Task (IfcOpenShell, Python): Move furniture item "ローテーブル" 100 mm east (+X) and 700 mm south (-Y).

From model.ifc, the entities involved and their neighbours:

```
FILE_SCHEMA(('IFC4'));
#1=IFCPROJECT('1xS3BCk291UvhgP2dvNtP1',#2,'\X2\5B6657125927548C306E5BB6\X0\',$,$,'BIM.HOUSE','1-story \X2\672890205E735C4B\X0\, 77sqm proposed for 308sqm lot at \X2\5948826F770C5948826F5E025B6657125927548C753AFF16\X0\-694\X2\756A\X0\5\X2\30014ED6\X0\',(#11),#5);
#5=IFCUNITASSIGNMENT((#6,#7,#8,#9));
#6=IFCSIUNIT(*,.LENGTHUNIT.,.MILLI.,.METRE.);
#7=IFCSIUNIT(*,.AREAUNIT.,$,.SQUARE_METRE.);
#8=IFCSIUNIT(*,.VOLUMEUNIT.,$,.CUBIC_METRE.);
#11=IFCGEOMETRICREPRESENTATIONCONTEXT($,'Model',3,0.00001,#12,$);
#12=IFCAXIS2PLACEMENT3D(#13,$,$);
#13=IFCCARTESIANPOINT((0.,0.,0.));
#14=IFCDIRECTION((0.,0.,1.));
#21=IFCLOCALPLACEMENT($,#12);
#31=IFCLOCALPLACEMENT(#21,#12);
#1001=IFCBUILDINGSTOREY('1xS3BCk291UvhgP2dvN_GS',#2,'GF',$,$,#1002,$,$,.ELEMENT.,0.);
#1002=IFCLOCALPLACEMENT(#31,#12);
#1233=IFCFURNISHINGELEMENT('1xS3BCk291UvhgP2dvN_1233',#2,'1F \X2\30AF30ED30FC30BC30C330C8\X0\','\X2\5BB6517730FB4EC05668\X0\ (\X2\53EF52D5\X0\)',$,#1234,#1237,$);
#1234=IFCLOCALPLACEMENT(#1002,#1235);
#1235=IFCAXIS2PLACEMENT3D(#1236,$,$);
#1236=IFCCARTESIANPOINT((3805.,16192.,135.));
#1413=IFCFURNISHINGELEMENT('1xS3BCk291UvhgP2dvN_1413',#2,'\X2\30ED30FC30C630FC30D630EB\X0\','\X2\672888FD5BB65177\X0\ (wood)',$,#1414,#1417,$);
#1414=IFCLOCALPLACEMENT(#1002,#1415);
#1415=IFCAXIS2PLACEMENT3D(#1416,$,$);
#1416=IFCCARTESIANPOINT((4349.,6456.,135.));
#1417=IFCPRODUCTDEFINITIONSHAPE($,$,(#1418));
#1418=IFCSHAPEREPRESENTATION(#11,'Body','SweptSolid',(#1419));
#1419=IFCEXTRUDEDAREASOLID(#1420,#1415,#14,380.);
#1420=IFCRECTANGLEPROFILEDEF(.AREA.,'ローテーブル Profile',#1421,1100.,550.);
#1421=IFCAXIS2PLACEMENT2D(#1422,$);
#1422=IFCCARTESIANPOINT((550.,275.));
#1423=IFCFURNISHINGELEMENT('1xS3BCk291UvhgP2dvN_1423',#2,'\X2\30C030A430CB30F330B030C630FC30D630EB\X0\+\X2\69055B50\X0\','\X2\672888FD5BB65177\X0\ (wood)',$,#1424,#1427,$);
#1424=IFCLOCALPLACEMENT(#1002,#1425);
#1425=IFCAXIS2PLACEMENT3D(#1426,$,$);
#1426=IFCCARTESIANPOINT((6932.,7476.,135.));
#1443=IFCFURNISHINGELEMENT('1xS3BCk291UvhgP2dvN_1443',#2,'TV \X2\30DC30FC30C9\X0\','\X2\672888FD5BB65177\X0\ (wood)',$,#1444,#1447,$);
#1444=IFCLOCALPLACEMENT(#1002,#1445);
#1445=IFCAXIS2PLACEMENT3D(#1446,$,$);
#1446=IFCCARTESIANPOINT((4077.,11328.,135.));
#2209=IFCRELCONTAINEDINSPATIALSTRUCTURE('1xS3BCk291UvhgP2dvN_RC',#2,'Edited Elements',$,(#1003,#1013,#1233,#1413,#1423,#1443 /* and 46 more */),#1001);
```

```python
import ifcopenshell
import ifcopenshell.api.geometry
import ifcopenshell.util.placement
import ifcopenshell.util.unit

model = ifcopenshell.open("model.ifc")
unit_scale = ifcopenshell.util.unit.calculate_unit_scale(model)

item = model.by_guid("1xS3BCk291UvhgP2dvN_1413")
matrix = ifcopenshell.util.placement.get_local_placement(item.ObjectPlacement)
matrix[0, 3] += 0.1 / unit_scale
matrix[1, 3] -= 0.7 / unit_scale
ifcopenshell.api.geometry.edit_object_placement(model, product=item, matrix=matrix, is_si=False)

print(ifcopenshell.util.placement.get_local_placement(item.ObjectPlacement).round(3) + 0.0)

model.write("model_edited.ifc")
```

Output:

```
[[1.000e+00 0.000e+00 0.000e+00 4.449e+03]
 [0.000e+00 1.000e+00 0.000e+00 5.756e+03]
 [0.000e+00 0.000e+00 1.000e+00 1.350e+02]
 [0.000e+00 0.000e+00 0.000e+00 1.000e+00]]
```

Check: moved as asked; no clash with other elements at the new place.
